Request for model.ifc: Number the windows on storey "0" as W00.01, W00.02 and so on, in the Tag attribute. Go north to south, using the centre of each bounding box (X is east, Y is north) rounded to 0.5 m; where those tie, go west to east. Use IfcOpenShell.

First a look at what the model holds.

```python
import ifcopenshell
import ifcopenshell.util.element
import ifcopenshell.util.placement

model = ifcopenshell.open("model.ifc")
print(model.schema)
storey = next(s for s in model.by_type("IfcBuildingStorey") if s.Name == "0")
windows = [e for e in ifcopenshell.util.element.get_decomposition(storey) if e.is_a("IfcWindow")]
for e in sorted(windows, key=lambda e: e.id()):
    origin = ifcopenshell.util.placement.get_local_placement(e.ObjectPlacement)[:3, 3]
    print(e.id(), e.Tag, e.Name, origin.round(2) + 0.0, sep=" | ")
```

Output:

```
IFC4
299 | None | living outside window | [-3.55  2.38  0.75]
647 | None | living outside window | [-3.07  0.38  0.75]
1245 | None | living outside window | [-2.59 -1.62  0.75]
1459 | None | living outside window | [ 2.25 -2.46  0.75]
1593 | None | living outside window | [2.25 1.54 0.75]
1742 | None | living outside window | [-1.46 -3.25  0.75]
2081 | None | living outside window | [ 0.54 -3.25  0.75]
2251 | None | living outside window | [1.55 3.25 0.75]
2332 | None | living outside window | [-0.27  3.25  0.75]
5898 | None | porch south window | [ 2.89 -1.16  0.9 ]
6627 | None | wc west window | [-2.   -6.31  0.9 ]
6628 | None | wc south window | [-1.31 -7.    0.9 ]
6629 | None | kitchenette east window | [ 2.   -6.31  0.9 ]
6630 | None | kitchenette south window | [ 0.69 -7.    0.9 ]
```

```python
import ifcopenshell
import ifcopenshell.geom
import ifcopenshell.util.element
import ifcopenshell.util.shape

model = ifcopenshell.open("model.ifc")
settings = ifcopenshell.geom.settings()
settings.set("use-world-coords", True)


def centre(element):
    shape = ifcopenshell.geom.create_shape(settings, element)
    return ifcopenshell.util.shape.get_bbox_centroid(shape.geometry)


storey = next(s for s in model.by_type("IfcBuildingStorey") if s.Name == "0")
windows = [e for e in ifcopenshell.util.element.get_decomposition(storey) if e.is_a("IfcWindow")]

# Insertion points can sit at a corner or the storey origin, so sort by the geometry (in metres).
centres = {e: centre(e) for e in windows}
windows.sort(key=lambda e: (-round(centres[e][1] / 0.5), centres[e][0]))

for i, e in enumerate(windows, start=1):
    number = f"W00.{i:02d}"
    e.Tag = number
    print(e.id(), number)

model.write("model_edited.ifc")
```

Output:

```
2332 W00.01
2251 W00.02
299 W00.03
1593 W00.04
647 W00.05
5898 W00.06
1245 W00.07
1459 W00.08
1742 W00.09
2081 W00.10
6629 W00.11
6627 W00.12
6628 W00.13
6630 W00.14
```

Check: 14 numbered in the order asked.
